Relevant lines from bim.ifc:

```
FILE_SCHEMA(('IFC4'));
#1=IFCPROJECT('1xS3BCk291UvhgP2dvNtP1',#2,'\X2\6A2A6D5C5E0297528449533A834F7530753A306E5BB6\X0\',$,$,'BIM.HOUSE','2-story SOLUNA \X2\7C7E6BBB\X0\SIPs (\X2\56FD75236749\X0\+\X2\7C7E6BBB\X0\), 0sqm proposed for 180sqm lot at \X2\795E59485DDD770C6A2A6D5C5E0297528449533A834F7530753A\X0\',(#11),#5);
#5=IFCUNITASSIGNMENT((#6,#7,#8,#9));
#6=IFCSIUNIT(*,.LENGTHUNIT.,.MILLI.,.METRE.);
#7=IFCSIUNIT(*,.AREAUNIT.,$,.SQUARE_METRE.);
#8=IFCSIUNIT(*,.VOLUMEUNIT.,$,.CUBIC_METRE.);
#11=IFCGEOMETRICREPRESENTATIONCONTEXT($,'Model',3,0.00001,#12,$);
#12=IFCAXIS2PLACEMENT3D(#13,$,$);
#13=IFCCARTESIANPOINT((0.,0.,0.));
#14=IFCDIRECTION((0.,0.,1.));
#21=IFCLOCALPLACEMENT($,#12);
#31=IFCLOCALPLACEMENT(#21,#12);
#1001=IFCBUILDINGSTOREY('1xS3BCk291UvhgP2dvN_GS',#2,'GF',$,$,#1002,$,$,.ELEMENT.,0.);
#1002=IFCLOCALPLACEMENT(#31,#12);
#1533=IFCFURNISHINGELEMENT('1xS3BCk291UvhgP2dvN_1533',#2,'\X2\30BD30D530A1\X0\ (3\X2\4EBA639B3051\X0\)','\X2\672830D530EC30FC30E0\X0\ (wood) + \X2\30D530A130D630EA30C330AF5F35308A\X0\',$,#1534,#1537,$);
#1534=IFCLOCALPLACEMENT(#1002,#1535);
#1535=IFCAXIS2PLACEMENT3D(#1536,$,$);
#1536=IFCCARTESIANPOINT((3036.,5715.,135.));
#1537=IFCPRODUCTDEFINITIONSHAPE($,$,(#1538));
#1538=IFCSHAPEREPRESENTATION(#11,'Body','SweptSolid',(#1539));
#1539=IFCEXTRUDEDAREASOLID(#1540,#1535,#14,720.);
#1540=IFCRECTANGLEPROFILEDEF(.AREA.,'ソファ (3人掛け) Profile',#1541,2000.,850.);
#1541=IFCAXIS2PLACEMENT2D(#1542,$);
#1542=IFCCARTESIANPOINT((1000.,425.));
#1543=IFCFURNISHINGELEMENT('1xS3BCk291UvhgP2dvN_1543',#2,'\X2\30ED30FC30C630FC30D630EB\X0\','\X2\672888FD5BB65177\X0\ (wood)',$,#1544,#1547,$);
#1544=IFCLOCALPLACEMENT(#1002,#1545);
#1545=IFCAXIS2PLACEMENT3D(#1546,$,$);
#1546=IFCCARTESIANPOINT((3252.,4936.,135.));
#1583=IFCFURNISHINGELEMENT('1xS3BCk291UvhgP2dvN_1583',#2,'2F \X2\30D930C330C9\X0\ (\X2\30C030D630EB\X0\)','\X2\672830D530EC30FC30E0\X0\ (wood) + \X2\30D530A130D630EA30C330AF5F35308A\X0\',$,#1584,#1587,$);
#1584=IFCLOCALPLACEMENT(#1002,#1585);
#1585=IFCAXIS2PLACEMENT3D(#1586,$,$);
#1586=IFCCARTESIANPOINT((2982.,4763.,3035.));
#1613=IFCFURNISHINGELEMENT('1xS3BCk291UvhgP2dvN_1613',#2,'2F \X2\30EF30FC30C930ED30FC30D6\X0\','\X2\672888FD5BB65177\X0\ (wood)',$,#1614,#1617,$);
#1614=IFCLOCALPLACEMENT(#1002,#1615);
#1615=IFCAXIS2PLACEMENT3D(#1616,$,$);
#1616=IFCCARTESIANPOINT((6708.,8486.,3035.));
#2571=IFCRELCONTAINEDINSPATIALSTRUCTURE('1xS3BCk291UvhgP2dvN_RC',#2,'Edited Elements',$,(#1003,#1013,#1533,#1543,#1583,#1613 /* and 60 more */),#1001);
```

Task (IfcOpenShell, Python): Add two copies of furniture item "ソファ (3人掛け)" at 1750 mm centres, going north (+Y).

```python
import numpy as np
import ifcopenshell
import ifcopenshell.api.geometry
import ifcopenshell.api.root
import ifcopenshell.util.element
import ifcopenshell.util.placement

model = ifcopenshell.open("bim.ifc")


def reuse_history(source, copy):
    """copy_class also copies each property set's owner history, people and application; keep the originals."""
    for rel in copy.IsDefinedBy:
        if rel.is_a("IfcRelDefinesByProperties") and (history := rel.RelatingPropertyDefinition.OwnerHistory):
            rel.RelatingPropertyDefinition.OwnerHistory = source.OwnerHistory
            ifcopenshell.util.element.remove_deep2(model, history)


source = model.by_guid("1xS3BCk291UvhgP2dvN_1533")
base = ifcopenshell.util.placement.get_local_placement(source.ObjectPlacement)
step = np.array([0.0, 1.0, 0.0]) * 1750.0

for i in range(1, 3):
    copy = ifcopenshell.api.root.copy_class(model, product=source)
    copy.Representation = ifcopenshell.util.element.copy_deep(
        model, source.Representation, exclude=["IfcGeometricRepresentationContext", "IfcRepresentationMap"]
    )
    reuse_history(source, copy)
    matrix = base.copy()
    matrix[:3, 3] += i * step
    print("added at", matrix[:3, 3].round(3) + 0.0)
    ifcopenshell.api.geometry.edit_object_placement(model, product=copy, matrix=matrix, is_si=False)

model.write("bim-out.ifc")
```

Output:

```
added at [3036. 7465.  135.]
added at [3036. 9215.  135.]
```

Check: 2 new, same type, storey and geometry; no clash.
